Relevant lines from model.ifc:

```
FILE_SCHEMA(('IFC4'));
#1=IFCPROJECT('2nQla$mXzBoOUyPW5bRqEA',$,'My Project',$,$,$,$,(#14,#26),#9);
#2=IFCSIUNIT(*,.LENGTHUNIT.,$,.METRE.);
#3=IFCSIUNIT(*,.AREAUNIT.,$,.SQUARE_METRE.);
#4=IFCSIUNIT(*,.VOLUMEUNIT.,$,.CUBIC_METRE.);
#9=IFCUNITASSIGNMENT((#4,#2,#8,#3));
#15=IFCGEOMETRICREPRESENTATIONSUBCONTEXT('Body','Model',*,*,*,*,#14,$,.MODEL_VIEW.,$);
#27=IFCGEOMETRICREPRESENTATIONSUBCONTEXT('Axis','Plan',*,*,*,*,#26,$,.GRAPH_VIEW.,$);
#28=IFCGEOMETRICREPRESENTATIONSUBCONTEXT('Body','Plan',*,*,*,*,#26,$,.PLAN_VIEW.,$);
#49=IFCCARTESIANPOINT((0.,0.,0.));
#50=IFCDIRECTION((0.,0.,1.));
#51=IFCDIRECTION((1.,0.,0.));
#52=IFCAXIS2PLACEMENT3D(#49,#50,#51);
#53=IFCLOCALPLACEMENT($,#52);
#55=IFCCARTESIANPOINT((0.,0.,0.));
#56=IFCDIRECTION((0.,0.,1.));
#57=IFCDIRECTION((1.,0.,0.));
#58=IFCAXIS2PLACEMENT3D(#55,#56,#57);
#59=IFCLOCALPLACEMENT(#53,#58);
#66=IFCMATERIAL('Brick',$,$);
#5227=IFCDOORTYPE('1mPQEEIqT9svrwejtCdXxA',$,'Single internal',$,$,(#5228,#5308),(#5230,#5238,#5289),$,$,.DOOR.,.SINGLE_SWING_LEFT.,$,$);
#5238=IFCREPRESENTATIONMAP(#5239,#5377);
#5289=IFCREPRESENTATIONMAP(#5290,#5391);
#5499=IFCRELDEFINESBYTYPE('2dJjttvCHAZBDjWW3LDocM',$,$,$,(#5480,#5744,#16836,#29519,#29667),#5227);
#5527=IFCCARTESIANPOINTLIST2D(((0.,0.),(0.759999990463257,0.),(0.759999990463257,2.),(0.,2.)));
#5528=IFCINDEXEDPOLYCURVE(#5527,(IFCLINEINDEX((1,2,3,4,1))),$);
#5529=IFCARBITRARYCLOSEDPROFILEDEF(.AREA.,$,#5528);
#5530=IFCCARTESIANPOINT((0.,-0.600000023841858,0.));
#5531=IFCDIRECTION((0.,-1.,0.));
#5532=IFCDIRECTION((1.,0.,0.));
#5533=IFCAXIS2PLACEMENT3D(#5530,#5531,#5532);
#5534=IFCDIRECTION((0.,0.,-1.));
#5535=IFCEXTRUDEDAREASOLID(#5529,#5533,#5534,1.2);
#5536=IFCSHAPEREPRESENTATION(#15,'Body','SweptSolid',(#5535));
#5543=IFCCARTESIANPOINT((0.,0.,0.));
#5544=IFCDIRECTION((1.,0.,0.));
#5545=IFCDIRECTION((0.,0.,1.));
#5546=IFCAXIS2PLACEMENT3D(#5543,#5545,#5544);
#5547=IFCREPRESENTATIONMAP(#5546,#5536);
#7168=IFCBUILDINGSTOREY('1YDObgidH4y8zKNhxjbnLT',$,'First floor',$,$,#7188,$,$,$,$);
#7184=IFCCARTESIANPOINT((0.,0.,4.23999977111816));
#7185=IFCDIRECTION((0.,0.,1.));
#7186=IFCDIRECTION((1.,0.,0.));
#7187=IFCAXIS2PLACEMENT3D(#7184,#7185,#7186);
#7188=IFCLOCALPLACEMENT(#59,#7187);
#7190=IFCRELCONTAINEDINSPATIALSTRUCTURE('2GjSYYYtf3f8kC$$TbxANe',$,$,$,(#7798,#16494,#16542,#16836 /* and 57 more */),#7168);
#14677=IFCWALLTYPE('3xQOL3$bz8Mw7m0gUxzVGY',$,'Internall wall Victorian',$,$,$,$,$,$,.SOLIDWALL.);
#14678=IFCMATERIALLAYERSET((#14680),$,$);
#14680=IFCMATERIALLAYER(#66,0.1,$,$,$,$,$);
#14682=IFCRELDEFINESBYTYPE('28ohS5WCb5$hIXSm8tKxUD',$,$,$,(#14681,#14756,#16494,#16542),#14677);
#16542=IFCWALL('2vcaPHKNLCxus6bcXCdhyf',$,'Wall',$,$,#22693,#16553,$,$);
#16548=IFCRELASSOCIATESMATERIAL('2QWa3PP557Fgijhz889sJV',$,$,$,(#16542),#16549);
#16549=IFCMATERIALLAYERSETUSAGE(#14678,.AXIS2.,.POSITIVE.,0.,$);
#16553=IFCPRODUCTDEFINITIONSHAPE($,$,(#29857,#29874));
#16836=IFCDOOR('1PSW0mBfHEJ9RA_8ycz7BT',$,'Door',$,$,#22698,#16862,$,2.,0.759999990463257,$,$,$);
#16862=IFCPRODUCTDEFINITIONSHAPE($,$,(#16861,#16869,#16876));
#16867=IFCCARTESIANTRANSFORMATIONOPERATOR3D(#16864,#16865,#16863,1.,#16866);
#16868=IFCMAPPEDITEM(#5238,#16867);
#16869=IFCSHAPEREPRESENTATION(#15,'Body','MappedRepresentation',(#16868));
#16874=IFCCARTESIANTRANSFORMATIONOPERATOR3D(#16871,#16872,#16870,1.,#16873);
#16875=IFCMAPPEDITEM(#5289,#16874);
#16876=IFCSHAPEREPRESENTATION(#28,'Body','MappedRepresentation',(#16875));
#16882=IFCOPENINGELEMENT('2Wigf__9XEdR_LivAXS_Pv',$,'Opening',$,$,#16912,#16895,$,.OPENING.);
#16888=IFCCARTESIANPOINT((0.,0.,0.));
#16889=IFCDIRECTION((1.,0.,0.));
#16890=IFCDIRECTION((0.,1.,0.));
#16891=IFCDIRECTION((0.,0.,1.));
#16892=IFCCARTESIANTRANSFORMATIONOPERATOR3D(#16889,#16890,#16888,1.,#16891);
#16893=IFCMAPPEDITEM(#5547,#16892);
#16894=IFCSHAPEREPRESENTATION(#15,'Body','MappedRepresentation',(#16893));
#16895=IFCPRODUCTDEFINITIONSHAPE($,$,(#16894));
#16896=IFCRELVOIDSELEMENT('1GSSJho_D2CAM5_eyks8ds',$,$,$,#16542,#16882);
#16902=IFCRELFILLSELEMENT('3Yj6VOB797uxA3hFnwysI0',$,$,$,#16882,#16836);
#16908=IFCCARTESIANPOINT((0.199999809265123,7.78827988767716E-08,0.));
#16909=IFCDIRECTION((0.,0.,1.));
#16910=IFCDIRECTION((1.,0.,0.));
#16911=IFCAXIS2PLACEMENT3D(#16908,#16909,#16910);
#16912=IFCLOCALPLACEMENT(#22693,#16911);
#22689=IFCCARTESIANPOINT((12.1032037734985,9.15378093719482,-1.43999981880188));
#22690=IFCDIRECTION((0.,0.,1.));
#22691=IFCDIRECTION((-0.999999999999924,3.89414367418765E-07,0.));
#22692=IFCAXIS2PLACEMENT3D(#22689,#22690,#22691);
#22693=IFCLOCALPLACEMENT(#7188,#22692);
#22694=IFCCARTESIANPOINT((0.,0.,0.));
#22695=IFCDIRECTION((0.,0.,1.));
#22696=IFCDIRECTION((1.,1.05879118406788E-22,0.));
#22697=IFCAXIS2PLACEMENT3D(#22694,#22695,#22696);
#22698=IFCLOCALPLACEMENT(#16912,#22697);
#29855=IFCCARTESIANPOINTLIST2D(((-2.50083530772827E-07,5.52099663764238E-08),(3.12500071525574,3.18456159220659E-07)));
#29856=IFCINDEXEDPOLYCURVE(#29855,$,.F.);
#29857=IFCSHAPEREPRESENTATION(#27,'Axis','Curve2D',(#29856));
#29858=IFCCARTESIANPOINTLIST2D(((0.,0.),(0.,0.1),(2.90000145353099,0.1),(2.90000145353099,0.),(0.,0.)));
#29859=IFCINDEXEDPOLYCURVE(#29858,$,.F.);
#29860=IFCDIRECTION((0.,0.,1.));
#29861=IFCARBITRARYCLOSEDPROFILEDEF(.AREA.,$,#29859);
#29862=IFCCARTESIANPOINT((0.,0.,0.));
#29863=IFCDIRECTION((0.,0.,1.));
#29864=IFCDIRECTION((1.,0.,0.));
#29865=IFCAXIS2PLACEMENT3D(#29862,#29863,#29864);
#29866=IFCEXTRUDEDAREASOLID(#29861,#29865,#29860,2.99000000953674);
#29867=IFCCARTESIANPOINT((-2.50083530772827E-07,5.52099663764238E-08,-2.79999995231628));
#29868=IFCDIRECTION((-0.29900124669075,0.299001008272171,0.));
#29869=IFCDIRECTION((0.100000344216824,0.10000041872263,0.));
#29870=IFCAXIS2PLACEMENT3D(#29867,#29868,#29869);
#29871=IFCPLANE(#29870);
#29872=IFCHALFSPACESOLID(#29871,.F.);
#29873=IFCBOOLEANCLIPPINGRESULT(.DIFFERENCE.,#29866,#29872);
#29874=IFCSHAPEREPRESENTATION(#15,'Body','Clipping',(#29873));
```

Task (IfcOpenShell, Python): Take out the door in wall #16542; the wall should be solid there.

```python
import ifcopenshell
import ifcopenshell.api.feature
import ifcopenshell.api.root
import ifcopenshell.geom
import ifcopenshell.util.shape

model = ifcopenshell.open("model.ifc")
settings = ifcopenshell.geom.settings()


def volume(element):
    """Net volume in cubic metres, openings subtracted."""
    shape = ifcopenshell.geom.create_shape(settings, element)
    return ifcopenshell.util.shape.get_volume(shape.geometry)


door = model.by_guid("1PSW0mBfHEJ9RA_8ycz7BT")
opening = door.FillsVoids[0].RelatingOpeningElement
wall = opening.VoidsElements[0].RelatingBuildingElement
before = volume(wall)

ifcopenshell.api.root.remove_product(model, product=door)
ifcopenshell.api.feature.remove_feature(model, feature=opening)

after = volume(wall)

print(f"wall volume {before:.3f} -> {after:.3f} m3")

model.write("model-out.ifc")
```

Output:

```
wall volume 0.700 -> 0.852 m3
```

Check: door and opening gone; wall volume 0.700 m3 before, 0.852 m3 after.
